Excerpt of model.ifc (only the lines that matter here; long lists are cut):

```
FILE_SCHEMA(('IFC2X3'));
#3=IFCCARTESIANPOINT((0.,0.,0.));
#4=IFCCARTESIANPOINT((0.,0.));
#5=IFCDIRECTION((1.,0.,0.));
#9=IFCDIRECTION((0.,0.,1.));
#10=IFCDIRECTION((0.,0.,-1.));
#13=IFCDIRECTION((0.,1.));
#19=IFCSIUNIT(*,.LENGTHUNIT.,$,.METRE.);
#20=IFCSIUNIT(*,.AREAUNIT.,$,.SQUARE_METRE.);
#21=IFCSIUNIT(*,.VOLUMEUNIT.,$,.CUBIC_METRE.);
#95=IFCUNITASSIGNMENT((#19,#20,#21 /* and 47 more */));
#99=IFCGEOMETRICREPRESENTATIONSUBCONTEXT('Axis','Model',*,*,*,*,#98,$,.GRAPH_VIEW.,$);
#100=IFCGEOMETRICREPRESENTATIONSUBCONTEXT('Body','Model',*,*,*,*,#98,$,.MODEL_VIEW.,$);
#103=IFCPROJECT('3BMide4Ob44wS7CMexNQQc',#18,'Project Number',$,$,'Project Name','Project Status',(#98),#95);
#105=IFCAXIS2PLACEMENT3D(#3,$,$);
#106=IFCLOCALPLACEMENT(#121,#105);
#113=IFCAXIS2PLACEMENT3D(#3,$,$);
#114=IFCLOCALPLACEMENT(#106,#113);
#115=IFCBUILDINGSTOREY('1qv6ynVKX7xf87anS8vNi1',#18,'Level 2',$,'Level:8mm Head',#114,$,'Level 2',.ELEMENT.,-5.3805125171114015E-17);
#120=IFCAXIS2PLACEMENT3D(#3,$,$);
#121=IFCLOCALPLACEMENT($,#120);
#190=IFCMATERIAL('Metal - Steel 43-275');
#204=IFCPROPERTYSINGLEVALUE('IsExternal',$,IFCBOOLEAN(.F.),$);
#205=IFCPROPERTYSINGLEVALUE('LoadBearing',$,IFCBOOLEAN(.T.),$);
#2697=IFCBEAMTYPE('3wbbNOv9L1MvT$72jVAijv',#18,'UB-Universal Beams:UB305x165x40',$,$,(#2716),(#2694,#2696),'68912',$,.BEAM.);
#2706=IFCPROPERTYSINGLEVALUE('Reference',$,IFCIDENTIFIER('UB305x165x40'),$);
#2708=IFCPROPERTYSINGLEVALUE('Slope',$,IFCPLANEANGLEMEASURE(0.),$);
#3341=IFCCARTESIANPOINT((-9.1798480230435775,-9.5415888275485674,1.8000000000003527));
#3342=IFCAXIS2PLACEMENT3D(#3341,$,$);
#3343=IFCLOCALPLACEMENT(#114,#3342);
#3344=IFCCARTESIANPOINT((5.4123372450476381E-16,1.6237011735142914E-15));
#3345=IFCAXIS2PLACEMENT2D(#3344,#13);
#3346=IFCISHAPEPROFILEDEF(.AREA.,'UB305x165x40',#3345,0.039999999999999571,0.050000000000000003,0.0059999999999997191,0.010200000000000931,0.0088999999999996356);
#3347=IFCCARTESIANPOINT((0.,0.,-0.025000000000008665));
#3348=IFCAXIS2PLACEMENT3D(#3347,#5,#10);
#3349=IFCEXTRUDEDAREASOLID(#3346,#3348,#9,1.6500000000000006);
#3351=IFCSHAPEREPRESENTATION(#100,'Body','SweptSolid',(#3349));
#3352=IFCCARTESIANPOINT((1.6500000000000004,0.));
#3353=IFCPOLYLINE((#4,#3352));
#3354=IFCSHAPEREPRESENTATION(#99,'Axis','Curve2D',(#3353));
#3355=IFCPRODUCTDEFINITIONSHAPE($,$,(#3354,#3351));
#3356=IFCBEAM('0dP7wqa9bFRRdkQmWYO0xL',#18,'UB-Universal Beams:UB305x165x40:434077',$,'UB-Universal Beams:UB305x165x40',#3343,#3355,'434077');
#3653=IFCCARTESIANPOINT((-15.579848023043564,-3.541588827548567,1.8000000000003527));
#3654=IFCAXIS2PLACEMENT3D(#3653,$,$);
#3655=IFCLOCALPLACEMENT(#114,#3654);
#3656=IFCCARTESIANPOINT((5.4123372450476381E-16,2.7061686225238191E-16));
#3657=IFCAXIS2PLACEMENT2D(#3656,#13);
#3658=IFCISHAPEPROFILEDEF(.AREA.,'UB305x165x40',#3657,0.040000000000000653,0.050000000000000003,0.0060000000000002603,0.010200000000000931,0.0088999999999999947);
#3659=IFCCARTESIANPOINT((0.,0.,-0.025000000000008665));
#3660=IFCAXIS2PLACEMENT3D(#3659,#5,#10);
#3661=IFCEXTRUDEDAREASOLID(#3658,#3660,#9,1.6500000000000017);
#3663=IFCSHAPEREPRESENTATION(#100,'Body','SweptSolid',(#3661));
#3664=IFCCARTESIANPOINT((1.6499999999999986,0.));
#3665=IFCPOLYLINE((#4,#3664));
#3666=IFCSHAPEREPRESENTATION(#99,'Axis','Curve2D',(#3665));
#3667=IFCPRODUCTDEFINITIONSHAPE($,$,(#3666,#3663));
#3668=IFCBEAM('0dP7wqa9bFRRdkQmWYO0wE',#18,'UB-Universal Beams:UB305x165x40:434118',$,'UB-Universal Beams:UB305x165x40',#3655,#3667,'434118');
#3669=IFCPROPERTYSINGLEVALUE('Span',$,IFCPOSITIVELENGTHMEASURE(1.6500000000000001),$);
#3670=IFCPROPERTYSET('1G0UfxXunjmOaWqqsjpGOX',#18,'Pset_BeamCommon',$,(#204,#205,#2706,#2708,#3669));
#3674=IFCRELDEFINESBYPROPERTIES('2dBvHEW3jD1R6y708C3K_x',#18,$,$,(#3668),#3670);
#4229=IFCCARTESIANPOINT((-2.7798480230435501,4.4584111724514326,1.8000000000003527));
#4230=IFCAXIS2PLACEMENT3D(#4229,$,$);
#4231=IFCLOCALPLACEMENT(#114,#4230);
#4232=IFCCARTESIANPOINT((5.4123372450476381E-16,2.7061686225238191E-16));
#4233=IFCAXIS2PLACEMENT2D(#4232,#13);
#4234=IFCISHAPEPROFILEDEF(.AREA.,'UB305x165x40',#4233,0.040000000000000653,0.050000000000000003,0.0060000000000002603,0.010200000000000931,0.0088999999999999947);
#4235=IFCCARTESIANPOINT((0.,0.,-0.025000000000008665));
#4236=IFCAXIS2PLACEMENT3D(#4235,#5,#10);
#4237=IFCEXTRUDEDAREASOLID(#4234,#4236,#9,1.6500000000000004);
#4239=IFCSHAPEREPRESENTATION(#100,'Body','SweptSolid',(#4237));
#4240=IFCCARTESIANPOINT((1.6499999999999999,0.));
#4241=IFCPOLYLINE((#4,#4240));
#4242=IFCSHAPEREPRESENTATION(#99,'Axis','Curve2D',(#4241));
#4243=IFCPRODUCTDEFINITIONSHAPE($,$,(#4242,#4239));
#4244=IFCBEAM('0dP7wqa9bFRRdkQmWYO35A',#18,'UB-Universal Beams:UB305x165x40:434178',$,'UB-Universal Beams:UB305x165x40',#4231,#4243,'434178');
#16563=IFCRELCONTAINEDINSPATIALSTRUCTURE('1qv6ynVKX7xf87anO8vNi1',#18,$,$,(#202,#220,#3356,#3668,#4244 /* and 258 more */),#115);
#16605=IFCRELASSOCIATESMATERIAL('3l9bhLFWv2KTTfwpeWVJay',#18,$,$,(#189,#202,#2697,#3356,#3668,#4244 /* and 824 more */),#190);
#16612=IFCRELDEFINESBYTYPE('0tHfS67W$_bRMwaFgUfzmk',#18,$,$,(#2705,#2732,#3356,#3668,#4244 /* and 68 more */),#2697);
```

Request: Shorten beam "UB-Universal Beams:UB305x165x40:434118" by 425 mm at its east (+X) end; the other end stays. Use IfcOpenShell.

```python
import numpy as np
import ifcopenshell
import ifcopenshell.api.pset
import ifcopenshell.util.element
import ifcopenshell.util.representation
import ifcopenshell.util.unit

model = ifcopenshell.open("model.ifc")
unit_scale = ifcopenshell.util.unit.calculate_unit_scale(model)

member = model.by_id(3668)
change = -0.425 / unit_scale

# The extrusion runs towards the end named, so only its depth changes.
body = ifcopenshell.util.representation.get_representation(member, "Model", "Body")
solid = body.Items[0]
old_length = solid.Depth
solid.Depth += change

# Move the axis end point with it.
axis = next(r for r in member.Representation.Representations if r.RepresentationIdentifier == "Axis").Items[0]
start, end = (np.array(p.Coordinates) for p in axis.Points)
end = end + (end - start) / np.linalg.norm(end - start) * change
point = model.createIfcCartesianPoint(end.tolist())
axis.Points = [axis.Points[0], point]

# Update the stored length and volume.
pset = model.by_id(ifcopenshell.util.element.get_pset(member, "Pset_BeamCommon", should_inherit=False)["id"])
ifcopenshell.api.pset.edit_pset(model, pset=pset, properties={
    "Span": model.create_entity("IfcPositiveLengthMeasure", solid.Depth),
})

print(f"length {old_length:g} -> {solid.Depth:g}")

model.write("model_rev.ifc")
```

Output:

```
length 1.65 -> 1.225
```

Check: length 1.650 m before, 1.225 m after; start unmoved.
